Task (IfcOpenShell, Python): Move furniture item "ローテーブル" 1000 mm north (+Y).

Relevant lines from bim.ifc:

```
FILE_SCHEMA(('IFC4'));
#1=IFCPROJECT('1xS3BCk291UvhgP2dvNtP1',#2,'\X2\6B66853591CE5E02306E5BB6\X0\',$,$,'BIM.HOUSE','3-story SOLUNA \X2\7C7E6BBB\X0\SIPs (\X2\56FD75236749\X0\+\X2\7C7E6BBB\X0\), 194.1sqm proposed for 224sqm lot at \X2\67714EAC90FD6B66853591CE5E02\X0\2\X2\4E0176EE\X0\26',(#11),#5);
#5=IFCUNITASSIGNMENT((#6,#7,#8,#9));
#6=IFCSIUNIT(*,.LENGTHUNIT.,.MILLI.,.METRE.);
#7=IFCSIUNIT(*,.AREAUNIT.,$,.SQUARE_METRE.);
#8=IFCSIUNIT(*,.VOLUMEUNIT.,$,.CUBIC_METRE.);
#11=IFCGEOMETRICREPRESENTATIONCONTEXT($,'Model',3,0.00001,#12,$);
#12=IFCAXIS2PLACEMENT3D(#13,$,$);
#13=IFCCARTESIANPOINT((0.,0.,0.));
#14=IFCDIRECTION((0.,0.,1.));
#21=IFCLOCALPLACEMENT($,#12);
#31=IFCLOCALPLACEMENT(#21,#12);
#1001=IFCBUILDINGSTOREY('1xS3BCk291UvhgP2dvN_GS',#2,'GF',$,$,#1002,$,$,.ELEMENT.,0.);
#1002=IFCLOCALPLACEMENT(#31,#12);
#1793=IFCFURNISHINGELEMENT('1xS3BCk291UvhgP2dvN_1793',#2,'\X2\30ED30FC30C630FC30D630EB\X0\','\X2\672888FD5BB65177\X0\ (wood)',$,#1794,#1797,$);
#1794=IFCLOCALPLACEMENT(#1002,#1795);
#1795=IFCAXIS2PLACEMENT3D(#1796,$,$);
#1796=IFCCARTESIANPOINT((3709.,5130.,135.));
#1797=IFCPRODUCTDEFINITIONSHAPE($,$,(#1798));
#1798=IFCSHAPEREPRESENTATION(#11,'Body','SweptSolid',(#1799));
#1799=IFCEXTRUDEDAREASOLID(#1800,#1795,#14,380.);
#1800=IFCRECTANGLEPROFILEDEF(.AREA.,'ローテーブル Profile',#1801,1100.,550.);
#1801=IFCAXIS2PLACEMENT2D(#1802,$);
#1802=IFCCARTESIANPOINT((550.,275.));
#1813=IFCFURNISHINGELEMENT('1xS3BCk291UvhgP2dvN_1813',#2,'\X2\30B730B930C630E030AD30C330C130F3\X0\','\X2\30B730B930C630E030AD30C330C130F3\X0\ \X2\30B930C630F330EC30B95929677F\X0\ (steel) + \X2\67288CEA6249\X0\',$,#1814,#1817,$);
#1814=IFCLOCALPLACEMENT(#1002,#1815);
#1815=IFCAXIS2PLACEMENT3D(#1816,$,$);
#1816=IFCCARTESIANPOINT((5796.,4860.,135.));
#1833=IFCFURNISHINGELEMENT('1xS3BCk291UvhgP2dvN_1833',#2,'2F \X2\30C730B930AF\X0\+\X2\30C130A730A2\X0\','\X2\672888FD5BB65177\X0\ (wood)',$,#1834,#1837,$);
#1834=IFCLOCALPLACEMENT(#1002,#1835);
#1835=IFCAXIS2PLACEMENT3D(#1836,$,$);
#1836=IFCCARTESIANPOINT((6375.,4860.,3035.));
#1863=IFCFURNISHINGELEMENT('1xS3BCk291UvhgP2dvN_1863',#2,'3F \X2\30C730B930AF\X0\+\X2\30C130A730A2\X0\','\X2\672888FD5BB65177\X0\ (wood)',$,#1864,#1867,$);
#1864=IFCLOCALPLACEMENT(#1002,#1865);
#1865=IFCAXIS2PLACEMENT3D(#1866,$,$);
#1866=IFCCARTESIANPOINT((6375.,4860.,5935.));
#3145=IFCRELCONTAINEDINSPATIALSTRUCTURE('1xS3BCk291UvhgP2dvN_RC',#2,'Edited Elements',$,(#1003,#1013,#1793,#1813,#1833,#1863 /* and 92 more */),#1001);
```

```python
import ifcopenshell
import ifcopenshell.api.geometry
import ifcopenshell.util.placement

model = ifcopenshell.open("bim.ifc")

item = model.by_guid("1xS3BCk291UvhgP2dvN_1793")
matrix = ifcopenshell.util.placement.get_local_placement(item.ObjectPlacement)
matrix[1, 3] += 1000.0
ifcopenshell.api.geometry.edit_object_placement(model, product=item, matrix=matrix, is_si=False)

print(ifcopenshell.util.placement.get_local_placement(item.ObjectPlacement).round(3) + 0.0)

model.write("bim_updated.ifc")
```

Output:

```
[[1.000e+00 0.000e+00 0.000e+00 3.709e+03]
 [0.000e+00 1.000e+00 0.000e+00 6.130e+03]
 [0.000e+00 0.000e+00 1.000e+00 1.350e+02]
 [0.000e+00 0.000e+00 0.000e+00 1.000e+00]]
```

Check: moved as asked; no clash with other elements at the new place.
